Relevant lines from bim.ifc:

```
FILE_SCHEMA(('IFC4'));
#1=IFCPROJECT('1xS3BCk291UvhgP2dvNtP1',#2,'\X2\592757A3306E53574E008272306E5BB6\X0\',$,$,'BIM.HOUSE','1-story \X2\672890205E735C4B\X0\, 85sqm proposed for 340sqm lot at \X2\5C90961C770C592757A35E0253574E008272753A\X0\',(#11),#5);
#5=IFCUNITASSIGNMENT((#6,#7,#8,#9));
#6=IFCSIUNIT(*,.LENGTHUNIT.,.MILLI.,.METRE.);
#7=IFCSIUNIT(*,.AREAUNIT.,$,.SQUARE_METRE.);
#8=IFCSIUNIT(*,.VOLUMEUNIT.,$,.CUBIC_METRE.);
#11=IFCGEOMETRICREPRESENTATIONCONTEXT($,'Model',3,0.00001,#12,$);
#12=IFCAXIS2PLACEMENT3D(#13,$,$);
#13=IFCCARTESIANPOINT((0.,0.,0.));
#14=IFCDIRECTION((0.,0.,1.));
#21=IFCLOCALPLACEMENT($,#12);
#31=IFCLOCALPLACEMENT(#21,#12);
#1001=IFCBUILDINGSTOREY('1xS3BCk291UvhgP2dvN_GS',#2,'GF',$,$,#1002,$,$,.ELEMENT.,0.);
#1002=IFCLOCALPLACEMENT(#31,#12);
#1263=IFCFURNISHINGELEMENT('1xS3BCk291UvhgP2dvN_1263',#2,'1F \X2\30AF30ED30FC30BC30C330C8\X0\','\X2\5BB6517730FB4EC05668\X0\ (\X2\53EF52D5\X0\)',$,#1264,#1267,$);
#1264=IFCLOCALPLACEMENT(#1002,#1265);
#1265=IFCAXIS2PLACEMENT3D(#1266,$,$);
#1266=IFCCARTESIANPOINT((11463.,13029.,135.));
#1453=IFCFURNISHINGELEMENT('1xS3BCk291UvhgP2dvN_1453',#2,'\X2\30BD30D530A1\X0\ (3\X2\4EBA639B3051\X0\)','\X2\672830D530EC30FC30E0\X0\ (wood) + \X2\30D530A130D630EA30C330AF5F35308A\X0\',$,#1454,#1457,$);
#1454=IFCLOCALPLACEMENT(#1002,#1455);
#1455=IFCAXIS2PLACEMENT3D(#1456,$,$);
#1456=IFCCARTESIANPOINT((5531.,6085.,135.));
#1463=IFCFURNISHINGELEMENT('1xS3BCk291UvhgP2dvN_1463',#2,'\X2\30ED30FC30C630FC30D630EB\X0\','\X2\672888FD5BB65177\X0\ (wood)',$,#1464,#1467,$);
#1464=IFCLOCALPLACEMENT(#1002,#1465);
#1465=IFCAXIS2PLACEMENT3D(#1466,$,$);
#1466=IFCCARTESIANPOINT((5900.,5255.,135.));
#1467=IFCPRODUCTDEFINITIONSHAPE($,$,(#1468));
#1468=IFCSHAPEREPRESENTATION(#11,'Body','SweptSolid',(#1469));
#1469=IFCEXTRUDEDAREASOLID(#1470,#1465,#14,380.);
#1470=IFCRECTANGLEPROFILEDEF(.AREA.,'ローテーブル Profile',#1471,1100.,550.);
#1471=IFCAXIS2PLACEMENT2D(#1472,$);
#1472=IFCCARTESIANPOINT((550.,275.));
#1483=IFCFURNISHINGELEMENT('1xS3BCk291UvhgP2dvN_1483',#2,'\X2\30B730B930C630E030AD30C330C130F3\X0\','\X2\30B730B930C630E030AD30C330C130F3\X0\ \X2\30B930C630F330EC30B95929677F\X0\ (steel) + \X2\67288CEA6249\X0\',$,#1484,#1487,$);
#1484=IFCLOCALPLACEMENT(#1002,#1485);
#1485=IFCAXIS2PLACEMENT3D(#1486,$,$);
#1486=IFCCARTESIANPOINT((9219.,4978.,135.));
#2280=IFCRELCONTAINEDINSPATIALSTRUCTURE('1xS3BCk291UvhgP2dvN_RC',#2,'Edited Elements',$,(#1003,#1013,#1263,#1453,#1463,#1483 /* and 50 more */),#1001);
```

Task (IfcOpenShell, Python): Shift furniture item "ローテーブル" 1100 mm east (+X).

```python
import ifcopenshell
import ifcopenshell.api.geometry
import ifcopenshell.util.placement
import ifcopenshell.util.unit

model = ifcopenshell.open("bim.ifc")
unit_scale = ifcopenshell.util.unit.calculate_unit_scale(model)

item = model.by_id(1463)
matrix = ifcopenshell.util.placement.get_local_placement(item.ObjectPlacement)
matrix[0, 3] += 1.1 / unit_scale
ifcopenshell.api.geometry.edit_object_placement(model, product=item, matrix=matrix, is_si=False)

print(ifcopenshell.util.placement.get_local_placement(item.ObjectPlacement).round(3) + 0.0)

model.write("bim_rev.ifc")
```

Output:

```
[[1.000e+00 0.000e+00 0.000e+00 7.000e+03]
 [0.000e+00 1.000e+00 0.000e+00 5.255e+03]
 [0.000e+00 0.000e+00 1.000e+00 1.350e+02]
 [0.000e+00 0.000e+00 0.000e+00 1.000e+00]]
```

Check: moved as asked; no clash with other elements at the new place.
